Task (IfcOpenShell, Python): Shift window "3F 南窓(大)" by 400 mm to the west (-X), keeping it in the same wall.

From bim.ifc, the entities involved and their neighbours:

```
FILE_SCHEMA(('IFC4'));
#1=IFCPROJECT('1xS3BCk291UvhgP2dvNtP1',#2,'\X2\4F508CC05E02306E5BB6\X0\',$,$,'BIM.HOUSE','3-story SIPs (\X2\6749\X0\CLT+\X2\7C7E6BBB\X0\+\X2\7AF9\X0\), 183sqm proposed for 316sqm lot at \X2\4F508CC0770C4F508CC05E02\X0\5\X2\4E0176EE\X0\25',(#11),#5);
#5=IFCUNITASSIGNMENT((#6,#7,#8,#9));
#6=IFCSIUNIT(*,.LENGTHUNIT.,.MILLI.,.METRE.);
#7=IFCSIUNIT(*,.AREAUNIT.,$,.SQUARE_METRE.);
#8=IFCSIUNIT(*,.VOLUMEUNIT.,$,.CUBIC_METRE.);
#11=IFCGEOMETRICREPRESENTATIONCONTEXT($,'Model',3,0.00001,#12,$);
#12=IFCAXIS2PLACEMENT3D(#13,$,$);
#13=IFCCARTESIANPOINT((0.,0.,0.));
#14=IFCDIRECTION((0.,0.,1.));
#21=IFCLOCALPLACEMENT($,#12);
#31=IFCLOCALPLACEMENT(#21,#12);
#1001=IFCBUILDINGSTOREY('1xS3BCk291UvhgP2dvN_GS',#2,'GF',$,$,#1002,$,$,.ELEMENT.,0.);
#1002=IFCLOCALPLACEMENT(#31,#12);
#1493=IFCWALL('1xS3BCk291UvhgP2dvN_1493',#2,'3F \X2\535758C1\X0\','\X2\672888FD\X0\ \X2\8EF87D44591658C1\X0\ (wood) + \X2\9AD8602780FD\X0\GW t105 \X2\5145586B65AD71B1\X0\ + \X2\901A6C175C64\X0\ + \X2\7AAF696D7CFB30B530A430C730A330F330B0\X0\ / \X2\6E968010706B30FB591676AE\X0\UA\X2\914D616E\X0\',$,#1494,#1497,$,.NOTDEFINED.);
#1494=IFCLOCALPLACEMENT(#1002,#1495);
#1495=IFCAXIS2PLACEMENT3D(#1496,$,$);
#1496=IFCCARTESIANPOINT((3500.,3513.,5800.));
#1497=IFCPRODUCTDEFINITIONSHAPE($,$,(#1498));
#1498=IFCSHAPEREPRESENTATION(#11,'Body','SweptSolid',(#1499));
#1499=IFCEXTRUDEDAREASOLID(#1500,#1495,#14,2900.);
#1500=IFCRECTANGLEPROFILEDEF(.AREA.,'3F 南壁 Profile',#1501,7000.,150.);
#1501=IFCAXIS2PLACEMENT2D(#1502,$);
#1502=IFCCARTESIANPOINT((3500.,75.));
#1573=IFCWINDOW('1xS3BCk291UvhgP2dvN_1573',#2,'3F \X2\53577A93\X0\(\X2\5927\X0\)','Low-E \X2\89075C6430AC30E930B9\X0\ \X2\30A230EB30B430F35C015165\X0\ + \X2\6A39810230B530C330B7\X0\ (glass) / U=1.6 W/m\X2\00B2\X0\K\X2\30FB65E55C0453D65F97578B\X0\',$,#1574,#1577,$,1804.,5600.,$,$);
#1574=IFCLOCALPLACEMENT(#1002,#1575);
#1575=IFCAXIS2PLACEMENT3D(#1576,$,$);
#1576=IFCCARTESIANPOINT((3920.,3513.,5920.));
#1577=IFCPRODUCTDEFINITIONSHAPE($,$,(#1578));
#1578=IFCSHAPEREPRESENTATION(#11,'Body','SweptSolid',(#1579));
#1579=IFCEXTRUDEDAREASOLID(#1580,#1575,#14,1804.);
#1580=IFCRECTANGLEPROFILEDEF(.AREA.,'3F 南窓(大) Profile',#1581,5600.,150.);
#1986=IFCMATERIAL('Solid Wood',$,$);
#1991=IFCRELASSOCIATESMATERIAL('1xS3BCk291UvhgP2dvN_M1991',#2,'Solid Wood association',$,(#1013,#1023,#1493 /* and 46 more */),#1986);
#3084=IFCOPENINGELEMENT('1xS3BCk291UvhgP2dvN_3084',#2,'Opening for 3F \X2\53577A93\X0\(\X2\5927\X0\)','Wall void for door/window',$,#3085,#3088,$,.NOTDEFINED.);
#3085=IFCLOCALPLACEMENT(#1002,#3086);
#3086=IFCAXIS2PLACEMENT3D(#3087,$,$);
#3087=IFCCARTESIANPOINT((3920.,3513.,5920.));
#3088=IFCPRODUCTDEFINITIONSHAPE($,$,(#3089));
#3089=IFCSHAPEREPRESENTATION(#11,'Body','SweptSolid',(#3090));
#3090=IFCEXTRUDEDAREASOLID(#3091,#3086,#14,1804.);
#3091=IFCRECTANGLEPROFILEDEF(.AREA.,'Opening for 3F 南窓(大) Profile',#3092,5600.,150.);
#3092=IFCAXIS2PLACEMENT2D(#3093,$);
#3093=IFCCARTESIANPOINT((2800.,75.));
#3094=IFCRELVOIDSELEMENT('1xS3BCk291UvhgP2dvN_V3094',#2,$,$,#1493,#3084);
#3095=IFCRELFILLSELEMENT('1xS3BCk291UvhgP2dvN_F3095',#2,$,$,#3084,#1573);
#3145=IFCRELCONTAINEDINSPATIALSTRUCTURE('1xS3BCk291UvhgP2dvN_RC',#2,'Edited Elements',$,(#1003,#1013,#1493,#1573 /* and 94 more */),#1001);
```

```python
import ifcopenshell
import ifcopenshell.api.geometry
import ifcopenshell.util.placement

model = ifcopenshell.open("bim.ifc")

window = model.by_guid("1xS3BCk291UvhgP2dvN_1573")
opening = window.FillsVoids[0].RelatingOpeningElement
wall = opening.VoidsElements[0].RelatingBuildingElement

wall_matrix = ifcopenshell.util.placement.get_local_placement(wall.ObjectPlacement)
shift = wall_matrix[:3, 0] * -400.0
before = ifcopenshell.util.placement.get_local_placement(window.ObjectPlacement)[:3, 3].copy()

# The window is not placed relative to its opening, so move both.
for product in (opening, window):
    matrix = ifcopenshell.util.placement.get_local_placement(product.ObjectPlacement)
    matrix[:3, 3] += shift
    ifcopenshell.api.geometry.edit_object_placement(model, product=product, matrix=matrix, is_si=False)

after = ifcopenshell.util.placement.get_local_placement(window.ObjectPlacement)[:3, 3]
print("window moved by", (after - before).round(3) + 0.0)

model.write("bim_updated.ifc")
```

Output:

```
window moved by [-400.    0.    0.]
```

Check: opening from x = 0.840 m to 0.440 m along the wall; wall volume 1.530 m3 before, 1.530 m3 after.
